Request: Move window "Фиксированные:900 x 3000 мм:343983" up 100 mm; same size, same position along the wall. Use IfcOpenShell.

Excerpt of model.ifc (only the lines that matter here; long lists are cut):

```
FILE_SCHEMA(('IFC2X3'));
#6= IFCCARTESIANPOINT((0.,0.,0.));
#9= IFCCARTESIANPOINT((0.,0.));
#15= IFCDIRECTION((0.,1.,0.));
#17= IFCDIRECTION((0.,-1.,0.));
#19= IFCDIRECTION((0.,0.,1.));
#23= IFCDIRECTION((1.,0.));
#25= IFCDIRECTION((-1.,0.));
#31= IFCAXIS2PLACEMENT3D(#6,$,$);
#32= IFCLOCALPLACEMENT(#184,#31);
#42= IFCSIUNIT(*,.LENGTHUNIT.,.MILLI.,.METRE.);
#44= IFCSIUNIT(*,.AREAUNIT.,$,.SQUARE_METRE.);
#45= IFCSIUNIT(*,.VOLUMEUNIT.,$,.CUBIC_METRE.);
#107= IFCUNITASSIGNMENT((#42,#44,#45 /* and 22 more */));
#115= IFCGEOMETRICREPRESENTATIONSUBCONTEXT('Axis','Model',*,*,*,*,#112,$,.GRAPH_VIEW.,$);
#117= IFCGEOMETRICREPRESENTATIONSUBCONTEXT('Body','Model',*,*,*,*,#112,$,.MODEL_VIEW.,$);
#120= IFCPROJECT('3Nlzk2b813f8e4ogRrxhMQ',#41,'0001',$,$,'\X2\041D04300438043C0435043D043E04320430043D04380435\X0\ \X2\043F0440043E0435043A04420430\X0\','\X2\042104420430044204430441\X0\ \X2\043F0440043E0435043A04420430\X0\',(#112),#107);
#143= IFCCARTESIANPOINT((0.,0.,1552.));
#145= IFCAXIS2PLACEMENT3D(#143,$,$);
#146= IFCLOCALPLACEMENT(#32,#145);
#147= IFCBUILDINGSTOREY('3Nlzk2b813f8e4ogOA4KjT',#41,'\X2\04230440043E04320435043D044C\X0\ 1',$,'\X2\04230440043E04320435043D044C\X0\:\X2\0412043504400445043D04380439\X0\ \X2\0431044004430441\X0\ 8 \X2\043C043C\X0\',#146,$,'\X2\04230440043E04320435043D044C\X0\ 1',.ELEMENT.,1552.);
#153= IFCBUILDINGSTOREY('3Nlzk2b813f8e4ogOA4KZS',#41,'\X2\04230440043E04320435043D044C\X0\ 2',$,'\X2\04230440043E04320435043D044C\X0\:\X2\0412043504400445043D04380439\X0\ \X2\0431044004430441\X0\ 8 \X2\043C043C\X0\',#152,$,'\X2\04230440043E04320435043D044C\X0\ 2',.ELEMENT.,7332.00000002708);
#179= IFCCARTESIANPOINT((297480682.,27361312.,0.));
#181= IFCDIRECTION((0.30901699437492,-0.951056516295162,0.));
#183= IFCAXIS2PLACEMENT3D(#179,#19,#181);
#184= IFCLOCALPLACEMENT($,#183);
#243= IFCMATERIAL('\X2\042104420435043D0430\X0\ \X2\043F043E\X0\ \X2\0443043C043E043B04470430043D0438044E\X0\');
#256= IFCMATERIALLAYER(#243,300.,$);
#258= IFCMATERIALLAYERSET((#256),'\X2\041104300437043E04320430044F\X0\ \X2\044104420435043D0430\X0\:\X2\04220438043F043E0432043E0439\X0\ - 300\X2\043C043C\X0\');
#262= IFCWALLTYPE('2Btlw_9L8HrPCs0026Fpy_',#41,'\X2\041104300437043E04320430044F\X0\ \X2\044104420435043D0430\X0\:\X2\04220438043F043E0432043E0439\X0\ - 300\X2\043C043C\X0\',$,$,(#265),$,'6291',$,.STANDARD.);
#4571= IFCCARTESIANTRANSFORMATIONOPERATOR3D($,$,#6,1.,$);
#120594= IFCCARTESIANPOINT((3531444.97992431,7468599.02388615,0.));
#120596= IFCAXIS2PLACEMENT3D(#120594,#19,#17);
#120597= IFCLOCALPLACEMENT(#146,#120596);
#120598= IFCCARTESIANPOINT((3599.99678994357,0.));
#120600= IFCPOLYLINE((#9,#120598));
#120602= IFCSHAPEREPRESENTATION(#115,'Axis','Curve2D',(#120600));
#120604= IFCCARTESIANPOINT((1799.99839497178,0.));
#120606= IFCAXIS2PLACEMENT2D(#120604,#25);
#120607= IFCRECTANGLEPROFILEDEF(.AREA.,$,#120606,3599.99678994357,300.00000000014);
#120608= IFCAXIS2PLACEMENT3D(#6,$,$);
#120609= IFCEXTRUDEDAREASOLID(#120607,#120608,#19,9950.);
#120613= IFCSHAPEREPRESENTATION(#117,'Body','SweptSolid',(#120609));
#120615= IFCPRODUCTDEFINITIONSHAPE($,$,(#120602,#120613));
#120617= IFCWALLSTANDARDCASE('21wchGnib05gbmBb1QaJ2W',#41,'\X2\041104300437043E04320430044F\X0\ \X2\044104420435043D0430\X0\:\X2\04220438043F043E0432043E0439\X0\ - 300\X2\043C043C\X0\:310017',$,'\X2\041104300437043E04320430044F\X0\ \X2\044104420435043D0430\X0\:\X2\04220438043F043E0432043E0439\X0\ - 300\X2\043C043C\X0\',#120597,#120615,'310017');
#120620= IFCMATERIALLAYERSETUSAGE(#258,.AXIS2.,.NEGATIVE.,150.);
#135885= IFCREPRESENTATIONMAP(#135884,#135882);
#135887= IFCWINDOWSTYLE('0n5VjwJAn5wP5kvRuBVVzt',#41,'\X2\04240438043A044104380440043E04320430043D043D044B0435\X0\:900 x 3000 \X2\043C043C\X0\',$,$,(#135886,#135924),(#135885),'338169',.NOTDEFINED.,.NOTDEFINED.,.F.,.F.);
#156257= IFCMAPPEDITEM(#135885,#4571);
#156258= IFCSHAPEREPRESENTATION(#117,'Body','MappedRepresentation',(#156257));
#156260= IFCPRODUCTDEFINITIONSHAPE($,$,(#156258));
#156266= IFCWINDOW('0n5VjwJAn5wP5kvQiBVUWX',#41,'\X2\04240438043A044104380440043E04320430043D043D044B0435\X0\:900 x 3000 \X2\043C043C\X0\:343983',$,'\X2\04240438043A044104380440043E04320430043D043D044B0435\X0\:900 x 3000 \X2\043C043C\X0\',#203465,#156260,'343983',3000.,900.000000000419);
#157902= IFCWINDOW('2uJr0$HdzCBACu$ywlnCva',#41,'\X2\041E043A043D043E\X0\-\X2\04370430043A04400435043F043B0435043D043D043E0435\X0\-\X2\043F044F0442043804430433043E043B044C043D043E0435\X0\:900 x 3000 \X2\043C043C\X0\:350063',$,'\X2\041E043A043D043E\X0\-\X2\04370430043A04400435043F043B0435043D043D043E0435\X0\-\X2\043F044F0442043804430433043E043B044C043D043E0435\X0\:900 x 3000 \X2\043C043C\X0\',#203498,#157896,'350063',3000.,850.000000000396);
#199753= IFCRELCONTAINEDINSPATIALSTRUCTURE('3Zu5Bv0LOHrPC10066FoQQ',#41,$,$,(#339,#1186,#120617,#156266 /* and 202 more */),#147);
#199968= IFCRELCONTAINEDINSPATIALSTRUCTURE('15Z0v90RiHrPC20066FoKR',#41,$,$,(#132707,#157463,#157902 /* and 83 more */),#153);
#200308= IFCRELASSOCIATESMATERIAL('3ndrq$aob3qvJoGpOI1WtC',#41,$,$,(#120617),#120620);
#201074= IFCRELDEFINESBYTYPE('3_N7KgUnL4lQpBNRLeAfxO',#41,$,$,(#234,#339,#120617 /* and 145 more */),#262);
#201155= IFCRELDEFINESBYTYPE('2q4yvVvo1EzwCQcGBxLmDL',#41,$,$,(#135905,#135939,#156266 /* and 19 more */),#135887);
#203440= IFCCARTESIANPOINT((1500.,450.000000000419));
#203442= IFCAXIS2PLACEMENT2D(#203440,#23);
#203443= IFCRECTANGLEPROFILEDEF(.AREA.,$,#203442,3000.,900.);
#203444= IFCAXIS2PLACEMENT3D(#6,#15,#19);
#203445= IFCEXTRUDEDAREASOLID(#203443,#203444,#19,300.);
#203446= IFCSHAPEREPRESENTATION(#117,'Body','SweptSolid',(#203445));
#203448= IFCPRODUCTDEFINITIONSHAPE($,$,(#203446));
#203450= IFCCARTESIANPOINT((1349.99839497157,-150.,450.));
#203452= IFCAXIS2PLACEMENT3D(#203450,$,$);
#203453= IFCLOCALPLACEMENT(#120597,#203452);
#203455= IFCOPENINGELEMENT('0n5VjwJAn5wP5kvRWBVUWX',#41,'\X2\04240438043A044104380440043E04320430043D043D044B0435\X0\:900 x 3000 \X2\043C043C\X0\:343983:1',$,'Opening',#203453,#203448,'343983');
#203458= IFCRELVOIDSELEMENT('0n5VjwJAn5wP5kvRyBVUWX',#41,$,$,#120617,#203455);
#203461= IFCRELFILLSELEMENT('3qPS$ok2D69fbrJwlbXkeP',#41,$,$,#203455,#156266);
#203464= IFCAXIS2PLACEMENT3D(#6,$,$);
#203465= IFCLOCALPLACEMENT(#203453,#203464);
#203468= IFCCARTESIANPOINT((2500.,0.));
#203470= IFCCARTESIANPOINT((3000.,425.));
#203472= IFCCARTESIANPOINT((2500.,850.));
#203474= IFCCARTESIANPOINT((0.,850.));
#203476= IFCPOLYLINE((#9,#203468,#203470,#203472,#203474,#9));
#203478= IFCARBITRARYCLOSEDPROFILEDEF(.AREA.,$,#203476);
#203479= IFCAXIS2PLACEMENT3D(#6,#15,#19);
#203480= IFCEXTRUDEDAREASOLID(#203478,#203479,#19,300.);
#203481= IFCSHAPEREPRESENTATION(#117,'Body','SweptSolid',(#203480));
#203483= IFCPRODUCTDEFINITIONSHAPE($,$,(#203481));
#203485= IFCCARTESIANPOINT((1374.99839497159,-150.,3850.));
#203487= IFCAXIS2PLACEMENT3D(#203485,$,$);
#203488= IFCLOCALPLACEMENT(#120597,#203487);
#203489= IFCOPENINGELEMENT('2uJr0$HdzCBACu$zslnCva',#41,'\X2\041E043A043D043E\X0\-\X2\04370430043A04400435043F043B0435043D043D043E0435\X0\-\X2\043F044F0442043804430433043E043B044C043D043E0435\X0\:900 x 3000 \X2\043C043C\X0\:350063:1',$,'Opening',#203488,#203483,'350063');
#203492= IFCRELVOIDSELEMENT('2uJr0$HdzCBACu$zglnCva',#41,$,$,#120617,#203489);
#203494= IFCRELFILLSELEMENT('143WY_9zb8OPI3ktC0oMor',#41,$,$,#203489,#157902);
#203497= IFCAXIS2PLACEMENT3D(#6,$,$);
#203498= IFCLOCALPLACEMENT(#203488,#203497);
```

```python
import numpy as np
import ifcopenshell
import ifcopenshell.api.geometry
import ifcopenshell.util.placement
import ifcopenshell.util.unit

model = ifcopenshell.open("model.ifc")
unit_scale = ifcopenshell.util.unit.calculate_unit_scale(model)

window = model.by_guid("0n5VjwJAn5wP5kvQiBVUWX")
opening = window.FillsVoids[0].RelatingOpeningElement
dz = 0.1 / unit_scale

shift = np.array([0.0, 0.0, dz])
# The window is placed relative to its opening, so it follows when the opening moves.
matrix = ifcopenshell.util.placement.get_local_placement(opening.ObjectPlacement)
matrix[:3, 3] += shift
ifcopenshell.api.geometry.edit_object_placement(
    model, product=opening, matrix=matrix, is_si=False, should_transform_children=True
)

print(f"moved by {dz * unit_scale:+.3f} m")

model.write("model_updated.ifc")
```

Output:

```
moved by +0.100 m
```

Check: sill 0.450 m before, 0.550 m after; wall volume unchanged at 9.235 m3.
